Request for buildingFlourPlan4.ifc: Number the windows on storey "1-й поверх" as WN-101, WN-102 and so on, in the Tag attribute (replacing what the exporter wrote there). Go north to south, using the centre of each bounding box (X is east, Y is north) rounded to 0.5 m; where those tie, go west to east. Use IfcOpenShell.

First a look at what the model holds.

```python
import ifcopenshell
import ifcopenshell.util.element
import ifcopenshell.util.placement

model = ifcopenshell.open("buildingFlourPlan4.ifc")
print(model.schema)
storey = next(s for s in model.by_type("IfcBuildingStorey") if s.Name == "1-й поверх")
windows = [e for e in ifcopenshell.util.element.get_decomposition(storey) if e.is_a("IfcWindow")]
for e in sorted(windows, key=lambda e: e.id()):
    origin = ifcopenshell.util.placement.get_local_placement(e.ObjectPlacement)[:3, 3]
    print(e.id(), e.Tag, e.Name, origin.round(2) + 0.0, sep=" | ")
```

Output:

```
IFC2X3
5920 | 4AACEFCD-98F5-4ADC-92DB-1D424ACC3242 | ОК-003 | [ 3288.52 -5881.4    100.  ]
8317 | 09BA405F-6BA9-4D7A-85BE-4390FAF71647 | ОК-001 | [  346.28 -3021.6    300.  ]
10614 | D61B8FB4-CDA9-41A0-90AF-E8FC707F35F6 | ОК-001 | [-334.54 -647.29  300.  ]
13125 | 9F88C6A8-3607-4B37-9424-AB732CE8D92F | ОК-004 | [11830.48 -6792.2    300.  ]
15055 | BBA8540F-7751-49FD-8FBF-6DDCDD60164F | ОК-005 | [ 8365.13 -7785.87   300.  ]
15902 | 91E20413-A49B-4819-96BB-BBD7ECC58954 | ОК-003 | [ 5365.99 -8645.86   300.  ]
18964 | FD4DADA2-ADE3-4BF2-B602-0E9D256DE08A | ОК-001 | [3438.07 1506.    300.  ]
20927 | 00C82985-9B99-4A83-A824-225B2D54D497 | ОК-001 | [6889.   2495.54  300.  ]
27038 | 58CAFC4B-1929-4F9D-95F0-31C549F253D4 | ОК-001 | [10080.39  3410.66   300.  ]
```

```python
import ifcopenshell
import ifcopenshell.geom
import ifcopenshell.util.element
import ifcopenshell.util.shape

model = ifcopenshell.open("buildingFlourPlan4.ifc")
settings = ifcopenshell.geom.settings()
settings.set("use-world-coords", True)


def centre(element):
    shape = ifcopenshell.geom.create_shape(settings, element)
    return ifcopenshell.util.shape.get_bbox_centroid(shape.geometry)


storey = next(s for s in model.by_type("IfcBuildingStorey") if s.Name == "1-й поверх")
windows = [e for e in ifcopenshell.util.element.get_decomposition(storey) if e.is_a("IfcWindow")]

# Insertion points can sit at a corner or the storey origin, so sort by the geometry (in metres).
centres = {e: centre(e) for e in windows}
windows.sort(key=lambda e: (-round(centres[e][1] / 0.5), centres[e][0]))

for i, e in enumerate(windows, start=1):
    number = f"WN-1{i:02d}"
    e.Tag = number
    print(e.id(), number)

model.write("buildingFlourPlan4_v2.ifc")
```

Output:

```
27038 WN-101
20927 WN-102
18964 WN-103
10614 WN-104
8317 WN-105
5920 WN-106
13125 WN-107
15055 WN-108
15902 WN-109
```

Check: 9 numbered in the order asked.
